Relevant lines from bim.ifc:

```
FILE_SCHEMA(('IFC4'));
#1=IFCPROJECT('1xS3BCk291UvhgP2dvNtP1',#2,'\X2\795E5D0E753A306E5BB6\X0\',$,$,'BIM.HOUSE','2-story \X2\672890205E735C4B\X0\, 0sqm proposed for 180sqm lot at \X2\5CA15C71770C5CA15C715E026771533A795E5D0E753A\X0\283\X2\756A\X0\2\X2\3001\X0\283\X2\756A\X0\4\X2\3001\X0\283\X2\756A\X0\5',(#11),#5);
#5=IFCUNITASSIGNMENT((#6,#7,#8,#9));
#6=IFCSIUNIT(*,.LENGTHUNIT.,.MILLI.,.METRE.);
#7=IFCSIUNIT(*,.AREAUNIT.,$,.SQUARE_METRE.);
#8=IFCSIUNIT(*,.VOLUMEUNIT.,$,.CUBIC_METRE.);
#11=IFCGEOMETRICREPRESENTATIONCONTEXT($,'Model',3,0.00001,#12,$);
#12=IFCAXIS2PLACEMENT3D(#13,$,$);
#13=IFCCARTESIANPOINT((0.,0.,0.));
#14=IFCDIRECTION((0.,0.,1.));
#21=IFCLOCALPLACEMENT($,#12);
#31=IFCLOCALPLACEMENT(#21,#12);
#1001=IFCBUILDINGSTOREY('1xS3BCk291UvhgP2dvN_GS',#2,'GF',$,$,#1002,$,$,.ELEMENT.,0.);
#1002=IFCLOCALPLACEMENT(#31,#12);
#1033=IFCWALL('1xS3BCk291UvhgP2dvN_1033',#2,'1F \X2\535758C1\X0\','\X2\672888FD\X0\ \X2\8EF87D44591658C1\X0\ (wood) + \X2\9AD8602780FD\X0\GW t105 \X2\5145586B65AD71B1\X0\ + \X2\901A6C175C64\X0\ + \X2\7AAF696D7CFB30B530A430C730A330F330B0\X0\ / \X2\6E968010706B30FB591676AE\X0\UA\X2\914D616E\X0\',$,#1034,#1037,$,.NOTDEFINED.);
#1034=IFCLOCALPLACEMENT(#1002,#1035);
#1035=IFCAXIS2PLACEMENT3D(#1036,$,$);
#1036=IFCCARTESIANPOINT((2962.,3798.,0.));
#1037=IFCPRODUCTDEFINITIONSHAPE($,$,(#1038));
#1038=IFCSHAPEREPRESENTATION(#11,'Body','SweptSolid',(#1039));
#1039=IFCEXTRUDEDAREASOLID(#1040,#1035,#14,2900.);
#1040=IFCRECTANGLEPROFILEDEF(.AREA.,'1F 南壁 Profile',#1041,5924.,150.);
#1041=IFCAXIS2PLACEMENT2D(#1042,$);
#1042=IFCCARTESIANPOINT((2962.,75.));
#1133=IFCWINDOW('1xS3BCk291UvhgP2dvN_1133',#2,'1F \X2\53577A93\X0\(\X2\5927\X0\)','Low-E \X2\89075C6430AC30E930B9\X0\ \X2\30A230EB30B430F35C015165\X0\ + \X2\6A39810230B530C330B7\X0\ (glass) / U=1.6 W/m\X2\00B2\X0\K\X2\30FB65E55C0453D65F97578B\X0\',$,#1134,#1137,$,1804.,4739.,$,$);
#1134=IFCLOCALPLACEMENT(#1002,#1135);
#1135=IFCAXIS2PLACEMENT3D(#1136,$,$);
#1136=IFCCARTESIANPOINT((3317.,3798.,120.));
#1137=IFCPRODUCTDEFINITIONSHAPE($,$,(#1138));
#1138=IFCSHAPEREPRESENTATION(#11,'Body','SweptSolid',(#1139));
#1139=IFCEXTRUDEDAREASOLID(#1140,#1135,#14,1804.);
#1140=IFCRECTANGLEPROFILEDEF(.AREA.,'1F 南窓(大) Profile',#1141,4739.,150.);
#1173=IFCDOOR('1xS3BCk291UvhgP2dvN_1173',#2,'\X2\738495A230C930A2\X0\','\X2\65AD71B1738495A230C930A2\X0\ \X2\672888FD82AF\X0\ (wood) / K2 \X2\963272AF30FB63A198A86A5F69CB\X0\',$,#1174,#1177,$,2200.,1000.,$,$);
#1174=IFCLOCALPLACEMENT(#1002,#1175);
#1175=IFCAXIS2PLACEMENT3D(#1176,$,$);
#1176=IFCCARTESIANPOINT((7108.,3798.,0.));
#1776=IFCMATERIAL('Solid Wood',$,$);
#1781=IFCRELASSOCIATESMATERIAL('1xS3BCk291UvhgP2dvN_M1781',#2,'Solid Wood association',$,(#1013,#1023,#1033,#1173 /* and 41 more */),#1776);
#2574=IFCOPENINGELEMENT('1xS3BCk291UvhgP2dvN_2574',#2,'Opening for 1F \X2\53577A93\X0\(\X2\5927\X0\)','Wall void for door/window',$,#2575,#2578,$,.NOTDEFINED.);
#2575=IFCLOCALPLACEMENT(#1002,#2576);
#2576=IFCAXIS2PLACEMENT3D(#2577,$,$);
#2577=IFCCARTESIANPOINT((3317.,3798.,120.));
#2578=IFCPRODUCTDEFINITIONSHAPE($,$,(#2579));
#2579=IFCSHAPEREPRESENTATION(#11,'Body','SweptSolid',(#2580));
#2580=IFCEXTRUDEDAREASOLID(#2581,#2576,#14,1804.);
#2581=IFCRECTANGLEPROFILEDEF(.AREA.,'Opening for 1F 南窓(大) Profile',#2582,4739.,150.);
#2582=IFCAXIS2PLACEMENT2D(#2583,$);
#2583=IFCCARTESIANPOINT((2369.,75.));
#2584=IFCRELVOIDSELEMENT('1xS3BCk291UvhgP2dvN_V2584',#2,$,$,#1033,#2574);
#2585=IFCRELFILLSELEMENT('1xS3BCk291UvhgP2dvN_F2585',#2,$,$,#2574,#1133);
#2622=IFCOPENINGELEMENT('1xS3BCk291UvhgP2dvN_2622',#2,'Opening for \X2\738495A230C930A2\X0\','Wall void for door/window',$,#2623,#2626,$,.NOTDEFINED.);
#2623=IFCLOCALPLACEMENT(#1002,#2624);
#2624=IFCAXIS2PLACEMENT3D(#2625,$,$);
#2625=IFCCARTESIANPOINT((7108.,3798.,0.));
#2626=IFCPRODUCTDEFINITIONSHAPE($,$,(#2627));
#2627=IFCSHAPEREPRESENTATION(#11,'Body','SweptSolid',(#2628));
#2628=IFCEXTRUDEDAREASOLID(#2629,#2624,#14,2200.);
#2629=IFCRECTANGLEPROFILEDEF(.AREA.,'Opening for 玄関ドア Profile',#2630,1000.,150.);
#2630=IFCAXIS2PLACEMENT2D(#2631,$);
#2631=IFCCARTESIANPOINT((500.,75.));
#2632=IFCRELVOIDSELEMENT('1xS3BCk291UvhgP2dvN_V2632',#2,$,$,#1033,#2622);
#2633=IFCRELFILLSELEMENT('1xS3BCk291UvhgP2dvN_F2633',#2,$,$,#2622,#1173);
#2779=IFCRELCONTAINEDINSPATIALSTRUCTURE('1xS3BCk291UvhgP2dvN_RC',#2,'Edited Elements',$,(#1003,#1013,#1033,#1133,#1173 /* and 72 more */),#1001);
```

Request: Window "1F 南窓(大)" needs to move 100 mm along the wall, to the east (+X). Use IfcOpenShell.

```python
import ifcopenshell
import ifcopenshell.api.geometry
import ifcopenshell.util.placement
import ifcopenshell.util.unit

model = ifcopenshell.open("bim.ifc")
unit_scale = ifcopenshell.util.unit.calculate_unit_scale(model)

window = model.by_id(1133)
opening = window.FillsVoids[0].RelatingOpeningElement
wall = opening.VoidsElements[0].RelatingBuildingElement

wall_matrix = ifcopenshell.util.placement.get_local_placement(wall.ObjectPlacement)
shift = wall_matrix[:3, 0] * 0.1 / unit_scale
before = ifcopenshell.util.placement.get_local_placement(window.ObjectPlacement)[:3, 3].copy()

# The window is not placed relative to its opening, so move both.
for product in (opening, window):
    matrix = ifcopenshell.util.placement.get_local_placement(product.ObjectPlacement)
    matrix[:3, 3] += shift
    ifcopenshell.api.geometry.edit_object_placement(model, product=product, matrix=matrix, is_si=False)

after = ifcopenshell.util.placement.get_local_placement(window.ObjectPlacement)[:3, 3]
print("window moved by", (after - before).round(3) + 0.0)

model.write("bim_updated.ifc")
```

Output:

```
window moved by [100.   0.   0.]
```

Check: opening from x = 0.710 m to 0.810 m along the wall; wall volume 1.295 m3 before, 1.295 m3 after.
